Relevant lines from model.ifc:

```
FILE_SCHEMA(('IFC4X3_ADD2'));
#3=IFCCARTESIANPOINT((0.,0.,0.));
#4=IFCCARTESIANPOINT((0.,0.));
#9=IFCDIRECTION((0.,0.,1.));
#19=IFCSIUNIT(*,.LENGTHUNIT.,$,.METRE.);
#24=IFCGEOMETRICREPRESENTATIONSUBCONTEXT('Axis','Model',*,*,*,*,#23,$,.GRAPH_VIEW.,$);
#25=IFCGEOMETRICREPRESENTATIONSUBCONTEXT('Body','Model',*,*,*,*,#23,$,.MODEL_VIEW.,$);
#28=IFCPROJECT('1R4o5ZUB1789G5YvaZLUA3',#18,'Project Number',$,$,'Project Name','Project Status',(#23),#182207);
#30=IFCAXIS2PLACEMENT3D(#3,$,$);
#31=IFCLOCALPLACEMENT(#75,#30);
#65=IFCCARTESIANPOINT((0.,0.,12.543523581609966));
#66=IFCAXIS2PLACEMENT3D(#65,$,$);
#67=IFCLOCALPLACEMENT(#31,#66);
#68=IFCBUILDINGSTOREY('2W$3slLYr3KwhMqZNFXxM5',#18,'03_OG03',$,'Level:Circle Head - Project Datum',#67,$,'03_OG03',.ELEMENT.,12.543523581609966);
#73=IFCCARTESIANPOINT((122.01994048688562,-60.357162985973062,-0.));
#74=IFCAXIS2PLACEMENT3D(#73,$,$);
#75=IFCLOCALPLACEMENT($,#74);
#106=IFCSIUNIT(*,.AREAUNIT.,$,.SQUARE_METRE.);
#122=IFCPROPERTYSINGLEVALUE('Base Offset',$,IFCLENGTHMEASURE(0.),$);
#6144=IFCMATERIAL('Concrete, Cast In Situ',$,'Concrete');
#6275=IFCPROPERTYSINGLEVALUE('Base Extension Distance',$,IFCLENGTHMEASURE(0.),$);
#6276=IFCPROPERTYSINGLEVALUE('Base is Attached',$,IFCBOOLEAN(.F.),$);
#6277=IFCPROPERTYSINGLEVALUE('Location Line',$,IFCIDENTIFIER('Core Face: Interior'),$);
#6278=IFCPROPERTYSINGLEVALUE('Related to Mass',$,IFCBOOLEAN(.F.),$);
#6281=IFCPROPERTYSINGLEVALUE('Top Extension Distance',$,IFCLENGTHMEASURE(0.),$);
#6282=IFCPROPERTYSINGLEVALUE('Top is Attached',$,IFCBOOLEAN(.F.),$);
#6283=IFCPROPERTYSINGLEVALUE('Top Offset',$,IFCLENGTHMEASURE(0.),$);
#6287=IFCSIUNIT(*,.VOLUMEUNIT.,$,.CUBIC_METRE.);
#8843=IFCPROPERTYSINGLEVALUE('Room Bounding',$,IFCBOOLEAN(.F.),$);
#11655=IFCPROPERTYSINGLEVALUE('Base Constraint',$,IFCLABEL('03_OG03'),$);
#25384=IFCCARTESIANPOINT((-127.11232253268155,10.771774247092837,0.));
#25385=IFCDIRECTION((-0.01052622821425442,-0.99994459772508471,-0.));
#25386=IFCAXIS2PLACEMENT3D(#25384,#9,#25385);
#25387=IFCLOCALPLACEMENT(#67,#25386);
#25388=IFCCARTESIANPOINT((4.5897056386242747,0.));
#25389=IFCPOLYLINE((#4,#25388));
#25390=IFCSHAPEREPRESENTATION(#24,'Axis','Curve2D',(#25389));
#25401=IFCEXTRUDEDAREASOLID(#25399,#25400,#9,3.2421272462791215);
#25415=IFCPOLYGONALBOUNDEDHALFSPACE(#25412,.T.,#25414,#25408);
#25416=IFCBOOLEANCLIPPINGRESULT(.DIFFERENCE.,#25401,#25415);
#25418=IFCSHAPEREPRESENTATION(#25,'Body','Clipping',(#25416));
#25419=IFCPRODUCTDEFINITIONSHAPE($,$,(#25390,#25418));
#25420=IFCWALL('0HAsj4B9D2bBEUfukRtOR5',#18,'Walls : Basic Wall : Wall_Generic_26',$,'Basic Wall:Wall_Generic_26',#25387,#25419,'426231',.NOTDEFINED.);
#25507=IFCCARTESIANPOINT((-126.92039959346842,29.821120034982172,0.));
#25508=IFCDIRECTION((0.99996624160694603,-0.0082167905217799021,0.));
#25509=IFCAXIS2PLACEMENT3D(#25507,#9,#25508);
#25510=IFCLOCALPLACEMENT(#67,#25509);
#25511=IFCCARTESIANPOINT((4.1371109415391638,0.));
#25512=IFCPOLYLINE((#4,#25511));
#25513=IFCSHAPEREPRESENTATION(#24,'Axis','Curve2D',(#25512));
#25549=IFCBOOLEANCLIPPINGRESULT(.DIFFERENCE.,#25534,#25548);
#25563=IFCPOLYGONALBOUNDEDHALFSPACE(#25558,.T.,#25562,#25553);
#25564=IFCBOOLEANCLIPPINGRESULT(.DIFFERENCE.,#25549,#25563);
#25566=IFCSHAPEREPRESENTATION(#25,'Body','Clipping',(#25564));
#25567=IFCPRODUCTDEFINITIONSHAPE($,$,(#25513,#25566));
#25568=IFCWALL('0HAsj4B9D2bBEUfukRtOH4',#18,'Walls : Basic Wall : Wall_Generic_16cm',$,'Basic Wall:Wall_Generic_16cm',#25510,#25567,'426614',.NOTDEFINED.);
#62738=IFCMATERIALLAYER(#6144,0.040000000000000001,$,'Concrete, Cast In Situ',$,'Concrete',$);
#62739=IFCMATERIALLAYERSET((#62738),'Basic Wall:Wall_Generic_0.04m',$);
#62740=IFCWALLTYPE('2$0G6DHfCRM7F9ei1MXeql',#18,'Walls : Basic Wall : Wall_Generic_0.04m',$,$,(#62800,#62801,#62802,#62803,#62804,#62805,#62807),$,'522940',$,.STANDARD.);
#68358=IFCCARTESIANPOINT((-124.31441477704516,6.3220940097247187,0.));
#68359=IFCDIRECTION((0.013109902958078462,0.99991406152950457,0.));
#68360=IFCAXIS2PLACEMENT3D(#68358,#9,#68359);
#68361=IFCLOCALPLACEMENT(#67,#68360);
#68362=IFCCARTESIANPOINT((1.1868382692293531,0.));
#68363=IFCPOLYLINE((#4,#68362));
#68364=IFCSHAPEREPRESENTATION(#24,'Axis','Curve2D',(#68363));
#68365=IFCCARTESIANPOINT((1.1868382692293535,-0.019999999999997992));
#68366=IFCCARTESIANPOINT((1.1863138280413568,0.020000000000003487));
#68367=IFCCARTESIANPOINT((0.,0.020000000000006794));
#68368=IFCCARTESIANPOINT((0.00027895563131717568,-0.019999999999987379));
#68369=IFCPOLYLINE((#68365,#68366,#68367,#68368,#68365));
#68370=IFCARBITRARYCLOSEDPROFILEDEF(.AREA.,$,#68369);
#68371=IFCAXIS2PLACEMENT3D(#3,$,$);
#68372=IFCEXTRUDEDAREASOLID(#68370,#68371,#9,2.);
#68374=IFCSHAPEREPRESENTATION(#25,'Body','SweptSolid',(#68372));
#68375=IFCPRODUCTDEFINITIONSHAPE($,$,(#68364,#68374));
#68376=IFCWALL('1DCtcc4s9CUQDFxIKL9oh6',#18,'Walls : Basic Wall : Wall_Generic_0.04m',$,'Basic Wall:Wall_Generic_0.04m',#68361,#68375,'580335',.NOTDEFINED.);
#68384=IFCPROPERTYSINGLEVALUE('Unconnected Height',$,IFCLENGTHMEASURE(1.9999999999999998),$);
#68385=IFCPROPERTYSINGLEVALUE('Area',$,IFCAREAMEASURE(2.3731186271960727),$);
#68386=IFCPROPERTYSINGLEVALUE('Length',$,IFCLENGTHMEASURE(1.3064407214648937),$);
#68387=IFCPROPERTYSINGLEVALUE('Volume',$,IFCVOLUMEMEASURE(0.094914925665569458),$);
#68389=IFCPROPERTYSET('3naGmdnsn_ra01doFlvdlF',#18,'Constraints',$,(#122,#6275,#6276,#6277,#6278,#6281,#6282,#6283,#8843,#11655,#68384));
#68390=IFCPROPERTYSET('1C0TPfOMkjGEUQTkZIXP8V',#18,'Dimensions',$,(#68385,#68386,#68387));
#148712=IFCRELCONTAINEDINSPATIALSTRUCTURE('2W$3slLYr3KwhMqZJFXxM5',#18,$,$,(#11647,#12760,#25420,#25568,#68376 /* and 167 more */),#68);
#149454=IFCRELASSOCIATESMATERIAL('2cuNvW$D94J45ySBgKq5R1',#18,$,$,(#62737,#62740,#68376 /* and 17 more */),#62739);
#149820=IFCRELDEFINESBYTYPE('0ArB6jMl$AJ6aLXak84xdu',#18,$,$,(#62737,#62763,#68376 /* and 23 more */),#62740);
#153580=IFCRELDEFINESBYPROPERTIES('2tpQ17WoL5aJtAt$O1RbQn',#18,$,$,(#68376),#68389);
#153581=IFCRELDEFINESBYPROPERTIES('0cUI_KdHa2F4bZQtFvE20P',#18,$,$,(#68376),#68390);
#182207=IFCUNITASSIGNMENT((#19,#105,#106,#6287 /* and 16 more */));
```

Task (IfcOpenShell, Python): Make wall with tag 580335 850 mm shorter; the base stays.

```python
import ifcopenshell
import ifcopenshell.api.pset
import ifcopenshell.geom
import ifcopenshell.util.element
import ifcopenshell.util.representation
import ifcopenshell.util.shape
import ifcopenshell.util.unit

model = ifcopenshell.open("model.ifc")
area_scale = ifcopenshell.util.unit.calculate_unit_scale(model, "AREAUNIT")
volume_scale = ifcopenshell.util.unit.calculate_unit_scale(model, "VOLUMEUNIT")
settings = ifcopenshell.geom.settings()


def volume(element):
    """Net volume in cubic metres, openings subtracted."""
    shape = ifcopenshell.geom.create_shape(settings, element)
    return ifcopenshell.util.shape.get_volume(shape.geometry)


wall = model.by_guid("1DCtcc4s9CUQDFxIKL9oh6")
before = volume(wall)

body = ifcopenshell.util.representation.get_representation(wall, "Model", "Body")
solid = body.Items[0]
old_height = solid.Depth
solid.Depth -= 0.85
after = volume(wall)
thickness = 0.04  # wall thickness in metres

# Update the stored height, areas and volumes.
pset = model.by_id(ifcopenshell.util.element.get_pset(wall, "Constraints", should_inherit=False)["id"])
ifcopenshell.api.pset.edit_pset(model, pset=pset, properties={
    "Unconnected Height": model.create_entity("IfcLengthMeasure", solid.Depth),
})
pset = model.by_id(ifcopenshell.util.element.get_pset(wall, "Dimensions", should_inherit=False)["id"])
ifcopenshell.api.pset.edit_pset(model, pset=pset, properties={
    "Area": model.create_entity("IfcAreaMeasure", after / thickness / area_scale),
    "Volume": model.create_entity("IfcVolumeMeasure", after / volume_scale),
})

print(f"height {old_height:g} -> {solid.Depth:g}, volume {before:.3f} -> {after:.3f} m3")

model.write("model-out.ifc")
```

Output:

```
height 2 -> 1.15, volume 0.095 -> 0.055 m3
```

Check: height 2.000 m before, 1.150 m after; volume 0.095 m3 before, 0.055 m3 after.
